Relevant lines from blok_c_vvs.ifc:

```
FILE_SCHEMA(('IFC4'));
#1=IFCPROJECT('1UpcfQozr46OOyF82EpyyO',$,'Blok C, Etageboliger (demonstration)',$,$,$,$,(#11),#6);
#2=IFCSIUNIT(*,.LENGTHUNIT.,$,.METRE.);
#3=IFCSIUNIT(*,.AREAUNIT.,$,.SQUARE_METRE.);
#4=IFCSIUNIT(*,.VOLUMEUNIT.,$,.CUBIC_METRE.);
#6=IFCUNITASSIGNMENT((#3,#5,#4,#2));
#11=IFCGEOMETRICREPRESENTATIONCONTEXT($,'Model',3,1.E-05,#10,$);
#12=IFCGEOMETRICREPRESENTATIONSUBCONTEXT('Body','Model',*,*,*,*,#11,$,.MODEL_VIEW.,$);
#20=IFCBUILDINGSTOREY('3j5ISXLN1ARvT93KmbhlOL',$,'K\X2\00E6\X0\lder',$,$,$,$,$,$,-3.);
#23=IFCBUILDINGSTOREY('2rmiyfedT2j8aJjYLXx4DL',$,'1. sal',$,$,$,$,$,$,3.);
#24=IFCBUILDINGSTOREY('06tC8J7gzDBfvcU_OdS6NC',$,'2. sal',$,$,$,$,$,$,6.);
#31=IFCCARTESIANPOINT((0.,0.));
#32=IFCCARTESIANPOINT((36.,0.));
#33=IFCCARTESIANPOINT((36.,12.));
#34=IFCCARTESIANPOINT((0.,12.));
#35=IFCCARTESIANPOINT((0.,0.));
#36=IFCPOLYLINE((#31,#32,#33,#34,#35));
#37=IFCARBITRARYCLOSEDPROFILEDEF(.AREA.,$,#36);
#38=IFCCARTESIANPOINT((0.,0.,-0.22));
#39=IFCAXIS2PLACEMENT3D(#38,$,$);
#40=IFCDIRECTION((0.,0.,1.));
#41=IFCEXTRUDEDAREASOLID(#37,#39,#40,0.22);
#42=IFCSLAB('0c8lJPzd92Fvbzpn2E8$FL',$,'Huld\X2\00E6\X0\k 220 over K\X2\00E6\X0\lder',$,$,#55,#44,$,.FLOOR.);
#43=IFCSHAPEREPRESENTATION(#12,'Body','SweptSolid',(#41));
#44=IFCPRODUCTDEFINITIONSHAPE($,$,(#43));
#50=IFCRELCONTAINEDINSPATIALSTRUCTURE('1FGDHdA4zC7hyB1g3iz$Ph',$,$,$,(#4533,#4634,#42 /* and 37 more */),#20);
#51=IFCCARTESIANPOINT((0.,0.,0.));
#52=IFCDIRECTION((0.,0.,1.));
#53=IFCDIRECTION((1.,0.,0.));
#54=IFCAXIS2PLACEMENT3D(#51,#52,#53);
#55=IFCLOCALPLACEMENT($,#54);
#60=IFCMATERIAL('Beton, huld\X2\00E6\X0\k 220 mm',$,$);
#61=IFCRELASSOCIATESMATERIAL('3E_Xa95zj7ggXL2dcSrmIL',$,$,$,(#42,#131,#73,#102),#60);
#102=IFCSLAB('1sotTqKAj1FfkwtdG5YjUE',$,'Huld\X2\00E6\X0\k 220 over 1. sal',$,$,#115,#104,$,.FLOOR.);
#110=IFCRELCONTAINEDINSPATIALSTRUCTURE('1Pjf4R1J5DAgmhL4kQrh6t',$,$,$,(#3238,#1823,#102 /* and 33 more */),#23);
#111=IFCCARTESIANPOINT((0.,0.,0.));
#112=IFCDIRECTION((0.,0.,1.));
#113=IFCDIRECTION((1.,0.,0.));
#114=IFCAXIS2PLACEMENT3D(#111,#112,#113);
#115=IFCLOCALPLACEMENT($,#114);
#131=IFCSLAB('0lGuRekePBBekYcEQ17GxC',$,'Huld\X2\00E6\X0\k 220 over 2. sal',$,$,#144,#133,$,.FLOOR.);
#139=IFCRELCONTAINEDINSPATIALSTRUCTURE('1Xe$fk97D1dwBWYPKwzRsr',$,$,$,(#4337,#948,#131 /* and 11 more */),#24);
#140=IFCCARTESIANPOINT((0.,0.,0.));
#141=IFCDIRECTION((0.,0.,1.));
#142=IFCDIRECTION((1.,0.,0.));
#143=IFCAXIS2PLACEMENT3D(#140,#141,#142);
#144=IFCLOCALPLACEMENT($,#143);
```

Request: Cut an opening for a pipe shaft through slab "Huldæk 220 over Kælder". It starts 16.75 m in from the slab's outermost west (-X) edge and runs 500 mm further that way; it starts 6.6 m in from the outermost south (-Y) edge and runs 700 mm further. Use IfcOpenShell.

```python
import numpy as np
import ifcopenshell
import ifcopenshell.api.feature
import ifcopenshell.api.geometry
import ifcopenshell.api.root
import ifcopenshell.geom
import ifcopenshell.util.placement
import ifcopenshell.util.representation
import ifcopenshell.util.shape
import ifcopenshell.util.unit

model = ifcopenshell.open("blok_c_vvs.ifc")
unit_scale = ifcopenshell.util.unit.calculate_unit_scale(model)
settings = ifcopenshell.geom.settings()


def volume(element):
    """Net volume in cubic metres, openings subtracted."""
    shape = ifcopenshell.geom.create_shape(settings, element)
    return ifcopenshell.util.shape.get_volume(shape.geometry)


slab = model.by_guid("0c8lJPzd92Fvbzpn2E8$FL")
before = volume(slab)

# Extent in the slab's own axes, in metres. The edges named are its -X and -Y sides.
slab_shape = ifcopenshell.geom.create_shape(settings, slab)
vertices = ifcopenshell.util.shape.get_vertices(slab_shape.geometry)
x_min, y_min, bottom = vertices.min(axis=0)
top = vertices[:, 2].max()

opening = ifcopenshell.api.root.create_entity(model, ifc_class="IfcOpeningElement", name="Pipe shaft opening", predefined_type="OPENING")
context = ifcopenshell.util.representation.get_context(model, "Model", "Body", "MODEL_VIEW")
width, depth = 0.5, 0.7
outline = [(0.0, 0.0), (width, 0.0), (width, depth), (0.0, depth), (0.0, 0.0)]
# Overshoot both faces by 50 mm so the cut is clean.
shape = ifcopenshell.api.geometry.add_slab_representation(
    model, context=context, depth=top - bottom + 0.1, polyline=outline
)
ifcopenshell.api.geometry.assign_representation(model, product=opening, representation=shape)

matrix = ifcopenshell.util.placement.get_local_placement(slab.ObjectPlacement)
matrix[:, 3] = matrix @ np.append(np.array([x_min + 16.75, y_min + 6.6, bottom - 0.05]) / unit_scale, 1.0)
ifcopenshell.api.geometry.edit_object_placement(model, product=opening, matrix=matrix, is_si=False)
ifcopenshell.api.feature.add_feature(model, feature=opening, element=slab)

after = volume(slab)

print(f"slab volume {before:.3f} -> {after:.3f} m3")

model.write("blok_c_vvs-out.ifc")
```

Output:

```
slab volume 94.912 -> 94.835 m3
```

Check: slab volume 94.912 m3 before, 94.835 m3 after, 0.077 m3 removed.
